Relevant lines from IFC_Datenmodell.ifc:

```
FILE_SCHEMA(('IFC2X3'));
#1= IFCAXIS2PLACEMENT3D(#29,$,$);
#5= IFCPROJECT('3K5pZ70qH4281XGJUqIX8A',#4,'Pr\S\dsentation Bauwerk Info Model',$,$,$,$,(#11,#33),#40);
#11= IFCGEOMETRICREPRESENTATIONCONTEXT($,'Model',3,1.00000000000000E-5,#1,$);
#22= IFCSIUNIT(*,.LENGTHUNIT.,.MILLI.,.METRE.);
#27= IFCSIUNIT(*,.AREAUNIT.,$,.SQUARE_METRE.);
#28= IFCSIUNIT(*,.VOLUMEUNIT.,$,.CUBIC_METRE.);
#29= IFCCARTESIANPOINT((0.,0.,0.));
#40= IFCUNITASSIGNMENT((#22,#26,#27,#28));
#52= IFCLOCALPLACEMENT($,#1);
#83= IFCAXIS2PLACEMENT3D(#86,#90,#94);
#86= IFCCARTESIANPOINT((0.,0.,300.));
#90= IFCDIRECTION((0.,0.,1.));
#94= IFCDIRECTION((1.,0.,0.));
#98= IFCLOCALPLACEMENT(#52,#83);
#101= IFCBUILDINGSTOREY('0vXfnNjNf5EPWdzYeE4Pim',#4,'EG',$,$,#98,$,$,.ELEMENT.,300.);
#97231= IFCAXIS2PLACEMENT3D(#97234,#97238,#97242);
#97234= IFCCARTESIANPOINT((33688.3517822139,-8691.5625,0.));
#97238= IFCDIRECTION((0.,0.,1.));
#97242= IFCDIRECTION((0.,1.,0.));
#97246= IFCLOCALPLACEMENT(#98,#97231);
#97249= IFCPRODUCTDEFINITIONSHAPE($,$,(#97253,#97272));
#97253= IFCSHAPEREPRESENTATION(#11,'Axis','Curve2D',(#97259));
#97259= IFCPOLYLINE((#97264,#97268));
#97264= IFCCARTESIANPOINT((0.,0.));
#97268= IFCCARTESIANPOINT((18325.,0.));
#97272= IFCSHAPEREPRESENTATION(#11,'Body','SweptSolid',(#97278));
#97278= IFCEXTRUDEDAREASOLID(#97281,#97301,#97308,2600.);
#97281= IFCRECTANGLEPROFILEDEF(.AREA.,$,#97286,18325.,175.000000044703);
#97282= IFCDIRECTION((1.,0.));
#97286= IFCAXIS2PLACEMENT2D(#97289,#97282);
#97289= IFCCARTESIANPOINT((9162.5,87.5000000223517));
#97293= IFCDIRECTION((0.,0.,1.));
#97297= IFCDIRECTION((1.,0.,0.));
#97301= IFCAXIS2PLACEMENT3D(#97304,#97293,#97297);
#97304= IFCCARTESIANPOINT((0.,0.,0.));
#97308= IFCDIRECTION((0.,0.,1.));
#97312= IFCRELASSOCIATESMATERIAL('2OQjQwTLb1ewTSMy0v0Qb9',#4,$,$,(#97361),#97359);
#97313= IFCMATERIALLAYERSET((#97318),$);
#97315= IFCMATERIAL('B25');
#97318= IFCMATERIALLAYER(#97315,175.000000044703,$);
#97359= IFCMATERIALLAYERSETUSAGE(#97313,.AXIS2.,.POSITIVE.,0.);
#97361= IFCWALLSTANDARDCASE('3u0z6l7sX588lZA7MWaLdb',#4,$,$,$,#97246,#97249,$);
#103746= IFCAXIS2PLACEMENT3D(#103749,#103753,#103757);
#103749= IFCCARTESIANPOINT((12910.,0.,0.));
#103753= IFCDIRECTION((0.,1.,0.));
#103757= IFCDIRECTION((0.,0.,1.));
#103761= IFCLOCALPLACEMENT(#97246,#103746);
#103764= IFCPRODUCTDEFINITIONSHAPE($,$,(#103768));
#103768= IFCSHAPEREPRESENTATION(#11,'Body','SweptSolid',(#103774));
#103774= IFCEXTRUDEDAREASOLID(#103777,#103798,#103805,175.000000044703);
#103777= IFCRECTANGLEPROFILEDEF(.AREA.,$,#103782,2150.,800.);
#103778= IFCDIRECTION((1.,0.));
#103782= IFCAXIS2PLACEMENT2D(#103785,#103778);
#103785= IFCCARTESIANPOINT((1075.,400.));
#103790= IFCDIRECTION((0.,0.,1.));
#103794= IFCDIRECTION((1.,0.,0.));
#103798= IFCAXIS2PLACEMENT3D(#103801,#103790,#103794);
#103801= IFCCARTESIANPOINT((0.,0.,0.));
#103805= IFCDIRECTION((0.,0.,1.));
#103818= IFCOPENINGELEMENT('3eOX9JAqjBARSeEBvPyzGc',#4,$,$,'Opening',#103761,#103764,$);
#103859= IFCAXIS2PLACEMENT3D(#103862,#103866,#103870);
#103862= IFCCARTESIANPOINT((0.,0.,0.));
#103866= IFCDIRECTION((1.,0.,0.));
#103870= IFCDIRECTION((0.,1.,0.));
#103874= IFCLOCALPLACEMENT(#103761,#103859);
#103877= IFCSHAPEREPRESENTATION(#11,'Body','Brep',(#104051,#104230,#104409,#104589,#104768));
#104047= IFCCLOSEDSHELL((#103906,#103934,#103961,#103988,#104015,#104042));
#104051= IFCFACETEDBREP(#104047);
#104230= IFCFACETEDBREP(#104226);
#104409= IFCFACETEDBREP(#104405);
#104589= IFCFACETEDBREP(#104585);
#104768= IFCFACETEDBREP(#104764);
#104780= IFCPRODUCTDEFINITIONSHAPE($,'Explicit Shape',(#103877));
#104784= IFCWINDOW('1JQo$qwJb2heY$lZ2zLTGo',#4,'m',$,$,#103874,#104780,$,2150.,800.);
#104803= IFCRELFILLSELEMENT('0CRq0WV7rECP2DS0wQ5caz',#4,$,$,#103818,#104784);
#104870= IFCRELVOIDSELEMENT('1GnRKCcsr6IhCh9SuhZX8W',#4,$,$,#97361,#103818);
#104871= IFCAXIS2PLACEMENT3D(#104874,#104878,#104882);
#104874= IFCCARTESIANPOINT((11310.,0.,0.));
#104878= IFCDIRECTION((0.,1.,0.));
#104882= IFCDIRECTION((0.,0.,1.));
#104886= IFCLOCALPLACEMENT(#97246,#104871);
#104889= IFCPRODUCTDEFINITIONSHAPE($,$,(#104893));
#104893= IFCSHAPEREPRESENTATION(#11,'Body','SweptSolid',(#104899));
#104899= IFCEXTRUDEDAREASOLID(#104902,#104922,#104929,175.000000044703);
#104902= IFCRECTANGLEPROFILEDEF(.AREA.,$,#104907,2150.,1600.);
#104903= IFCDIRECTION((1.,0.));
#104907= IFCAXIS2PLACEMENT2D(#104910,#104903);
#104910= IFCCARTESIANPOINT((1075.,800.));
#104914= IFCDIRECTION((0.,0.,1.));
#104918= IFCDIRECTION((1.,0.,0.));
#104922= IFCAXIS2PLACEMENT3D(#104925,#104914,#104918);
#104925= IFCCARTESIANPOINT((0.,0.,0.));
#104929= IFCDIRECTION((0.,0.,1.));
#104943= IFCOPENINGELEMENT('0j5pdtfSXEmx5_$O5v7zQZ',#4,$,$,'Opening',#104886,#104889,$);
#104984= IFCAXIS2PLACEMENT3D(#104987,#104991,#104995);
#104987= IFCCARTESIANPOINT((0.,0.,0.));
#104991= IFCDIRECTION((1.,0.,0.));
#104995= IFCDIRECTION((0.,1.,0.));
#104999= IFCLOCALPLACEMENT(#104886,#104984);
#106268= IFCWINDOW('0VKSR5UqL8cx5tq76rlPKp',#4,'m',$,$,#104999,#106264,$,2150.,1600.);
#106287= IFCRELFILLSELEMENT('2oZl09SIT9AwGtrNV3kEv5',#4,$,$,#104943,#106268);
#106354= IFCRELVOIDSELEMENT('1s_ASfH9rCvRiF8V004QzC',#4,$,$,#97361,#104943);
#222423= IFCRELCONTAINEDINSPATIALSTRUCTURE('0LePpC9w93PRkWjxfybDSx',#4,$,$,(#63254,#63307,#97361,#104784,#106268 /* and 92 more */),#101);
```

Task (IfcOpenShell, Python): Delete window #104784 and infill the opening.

```python
import ifcopenshell
import ifcopenshell.api.feature
import ifcopenshell.api.root
import ifcopenshell.geom
import ifcopenshell.util.shape

model = ifcopenshell.open("IFC_Datenmodell.ifc")
settings = ifcopenshell.geom.settings()


def volume(element):
    """Net volume in cubic metres, openings subtracted."""
    shape = ifcopenshell.geom.create_shape(settings, element)
    return ifcopenshell.util.shape.get_volume(shape.geometry)


window = model.by_guid("1JQo$qwJb2heY$lZ2zLTGo")
opening = window.FillsVoids[0].RelatingOpeningElement
wall = opening.VoidsElements[0].RelatingBuildingElement
before = volume(wall)

ifcopenshell.api.root.remove_product(model, product=window)
ifcopenshell.api.feature.remove_feature(model, feature=opening)

after = volume(wall)

print(f"wall volume {before:.3f} -> {after:.3f} m3")

model.write("IFC_Datenmodell_rev.ifc")
```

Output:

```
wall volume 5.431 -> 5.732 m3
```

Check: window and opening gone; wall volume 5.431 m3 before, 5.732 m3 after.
